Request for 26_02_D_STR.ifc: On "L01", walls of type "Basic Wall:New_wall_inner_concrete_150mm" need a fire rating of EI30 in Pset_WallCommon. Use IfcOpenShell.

First a look at what the model holds.

```python
import ifcopenshell
import ifcopenshell.util.element

model = ifcopenshell.open("26_02_D_STR.ifc")
print(model.schema)
storey = next(s for s in model.by_type("IfcBuildingStorey") if s.Name == "L01")
walls = [e for e in ifcopenshell.util.element.get_decomposition(storey) if e.is_a("IfcWall")]
seen = {}
for e in walls:
    element_type = ifcopenshell.util.element.get_type(e)
    key = (element_type.Name if element_type != e and element_type else None, ifcopenshell.util.element.get_pset(e, "Pset_WallCommon", "FireRating"))
    seen[key] = seen.get(key, 0) + 1
for (name, value), count in sorted(seen.items(), key=str):
    print(count, "x", name, "|", value)
```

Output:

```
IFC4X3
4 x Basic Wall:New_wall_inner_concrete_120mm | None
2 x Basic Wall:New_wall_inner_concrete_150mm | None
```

```python
import ifcopenshell
import ifcopenshell.api.pset
import ifcopenshell.util.element

model = ifcopenshell.open("26_02_D_STR.ifc")

storey = next(s for s in model.by_type("IfcBuildingStorey") if s.Name == "L01")
walls = [e for e in ifcopenshell.util.element.get_decomposition(storey) if e.is_a("IfcWall")]

count = 0
for e in walls:
    element_type = ifcopenshell.util.element.get_type(e)
    if element_type in (None, e) or element_type.Name != "Basic Wall:New_wall_inner_concrete_150mm":
        continue
    # add_pset returns the element's existing set when there is one.
    pset = ifcopenshell.api.pset.add_pset(model, product=e, name="Pset_WallCommon")
    ifcopenshell.api.pset.edit_pset(model, pset=pset, properties={"FireRating": "EI30"})
    count += 1

print(count, "walls updated")

model.write("26_02_D_STR_v2.ifc")
```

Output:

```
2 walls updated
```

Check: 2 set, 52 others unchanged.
